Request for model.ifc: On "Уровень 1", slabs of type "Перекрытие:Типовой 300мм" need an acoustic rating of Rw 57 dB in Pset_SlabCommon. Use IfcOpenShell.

First a look at what the model holds.

```python
import ifcopenshell
import ifcopenshell.util.element

model = ifcopenshell.open("model.ifc")
print(model.schema)
storey = next(s for s in model.by_type("IfcBuildingStorey") if s.Name == "Уровень 1")
slabs = [e for e in ifcopenshell.util.element.get_decomposition(storey) if e.is_a("IfcSlab")]
seen = {}
for e in slabs:
    element_type = ifcopenshell.util.element.get_type(e)
    key = (element_type.Name if element_type != e and element_type else None, ifcopenshell.util.element.get_pset(e, "Pset_SlabCommon", "AcousticRating"))
    seen[key] = seen.get(key, 0) + 1
for (name, value), count in sorted(seen.items(), key=str):
    print(count, "x", name, "|", value)
```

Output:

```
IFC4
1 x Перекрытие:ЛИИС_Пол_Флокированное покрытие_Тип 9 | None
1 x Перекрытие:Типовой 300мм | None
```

```python
import ifcopenshell
import ifcopenshell.api.pset
import ifcopenshell.util.element

model = ifcopenshell.open("model.ifc")

storey = next(s for s in model.by_type("IfcBuildingStorey") if s.Name == "Уровень 1")
slabs = [e for e in ifcopenshell.util.element.get_decomposition(storey) if e.is_a("IfcSlab")]

count = 0
for e in slabs:
    element_type = ifcopenshell.util.element.get_type(e)
    if element_type in (None, e) or element_type.Name != "Перекрытие:Типовой 300мм":
        continue
    # add_pset returns the element's existing set when there is one.
    pset = ifcopenshell.api.pset.add_pset(model, product=e, name="Pset_SlabCommon")
    ifcopenshell.api.pset.edit_pset(model, pset=pset, properties={"AcousticRating": "Rw 57 dB"})
    count += 1

print(count, "slabs updated")

model.write("model_edited.ifc")
```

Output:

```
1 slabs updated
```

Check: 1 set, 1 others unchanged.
